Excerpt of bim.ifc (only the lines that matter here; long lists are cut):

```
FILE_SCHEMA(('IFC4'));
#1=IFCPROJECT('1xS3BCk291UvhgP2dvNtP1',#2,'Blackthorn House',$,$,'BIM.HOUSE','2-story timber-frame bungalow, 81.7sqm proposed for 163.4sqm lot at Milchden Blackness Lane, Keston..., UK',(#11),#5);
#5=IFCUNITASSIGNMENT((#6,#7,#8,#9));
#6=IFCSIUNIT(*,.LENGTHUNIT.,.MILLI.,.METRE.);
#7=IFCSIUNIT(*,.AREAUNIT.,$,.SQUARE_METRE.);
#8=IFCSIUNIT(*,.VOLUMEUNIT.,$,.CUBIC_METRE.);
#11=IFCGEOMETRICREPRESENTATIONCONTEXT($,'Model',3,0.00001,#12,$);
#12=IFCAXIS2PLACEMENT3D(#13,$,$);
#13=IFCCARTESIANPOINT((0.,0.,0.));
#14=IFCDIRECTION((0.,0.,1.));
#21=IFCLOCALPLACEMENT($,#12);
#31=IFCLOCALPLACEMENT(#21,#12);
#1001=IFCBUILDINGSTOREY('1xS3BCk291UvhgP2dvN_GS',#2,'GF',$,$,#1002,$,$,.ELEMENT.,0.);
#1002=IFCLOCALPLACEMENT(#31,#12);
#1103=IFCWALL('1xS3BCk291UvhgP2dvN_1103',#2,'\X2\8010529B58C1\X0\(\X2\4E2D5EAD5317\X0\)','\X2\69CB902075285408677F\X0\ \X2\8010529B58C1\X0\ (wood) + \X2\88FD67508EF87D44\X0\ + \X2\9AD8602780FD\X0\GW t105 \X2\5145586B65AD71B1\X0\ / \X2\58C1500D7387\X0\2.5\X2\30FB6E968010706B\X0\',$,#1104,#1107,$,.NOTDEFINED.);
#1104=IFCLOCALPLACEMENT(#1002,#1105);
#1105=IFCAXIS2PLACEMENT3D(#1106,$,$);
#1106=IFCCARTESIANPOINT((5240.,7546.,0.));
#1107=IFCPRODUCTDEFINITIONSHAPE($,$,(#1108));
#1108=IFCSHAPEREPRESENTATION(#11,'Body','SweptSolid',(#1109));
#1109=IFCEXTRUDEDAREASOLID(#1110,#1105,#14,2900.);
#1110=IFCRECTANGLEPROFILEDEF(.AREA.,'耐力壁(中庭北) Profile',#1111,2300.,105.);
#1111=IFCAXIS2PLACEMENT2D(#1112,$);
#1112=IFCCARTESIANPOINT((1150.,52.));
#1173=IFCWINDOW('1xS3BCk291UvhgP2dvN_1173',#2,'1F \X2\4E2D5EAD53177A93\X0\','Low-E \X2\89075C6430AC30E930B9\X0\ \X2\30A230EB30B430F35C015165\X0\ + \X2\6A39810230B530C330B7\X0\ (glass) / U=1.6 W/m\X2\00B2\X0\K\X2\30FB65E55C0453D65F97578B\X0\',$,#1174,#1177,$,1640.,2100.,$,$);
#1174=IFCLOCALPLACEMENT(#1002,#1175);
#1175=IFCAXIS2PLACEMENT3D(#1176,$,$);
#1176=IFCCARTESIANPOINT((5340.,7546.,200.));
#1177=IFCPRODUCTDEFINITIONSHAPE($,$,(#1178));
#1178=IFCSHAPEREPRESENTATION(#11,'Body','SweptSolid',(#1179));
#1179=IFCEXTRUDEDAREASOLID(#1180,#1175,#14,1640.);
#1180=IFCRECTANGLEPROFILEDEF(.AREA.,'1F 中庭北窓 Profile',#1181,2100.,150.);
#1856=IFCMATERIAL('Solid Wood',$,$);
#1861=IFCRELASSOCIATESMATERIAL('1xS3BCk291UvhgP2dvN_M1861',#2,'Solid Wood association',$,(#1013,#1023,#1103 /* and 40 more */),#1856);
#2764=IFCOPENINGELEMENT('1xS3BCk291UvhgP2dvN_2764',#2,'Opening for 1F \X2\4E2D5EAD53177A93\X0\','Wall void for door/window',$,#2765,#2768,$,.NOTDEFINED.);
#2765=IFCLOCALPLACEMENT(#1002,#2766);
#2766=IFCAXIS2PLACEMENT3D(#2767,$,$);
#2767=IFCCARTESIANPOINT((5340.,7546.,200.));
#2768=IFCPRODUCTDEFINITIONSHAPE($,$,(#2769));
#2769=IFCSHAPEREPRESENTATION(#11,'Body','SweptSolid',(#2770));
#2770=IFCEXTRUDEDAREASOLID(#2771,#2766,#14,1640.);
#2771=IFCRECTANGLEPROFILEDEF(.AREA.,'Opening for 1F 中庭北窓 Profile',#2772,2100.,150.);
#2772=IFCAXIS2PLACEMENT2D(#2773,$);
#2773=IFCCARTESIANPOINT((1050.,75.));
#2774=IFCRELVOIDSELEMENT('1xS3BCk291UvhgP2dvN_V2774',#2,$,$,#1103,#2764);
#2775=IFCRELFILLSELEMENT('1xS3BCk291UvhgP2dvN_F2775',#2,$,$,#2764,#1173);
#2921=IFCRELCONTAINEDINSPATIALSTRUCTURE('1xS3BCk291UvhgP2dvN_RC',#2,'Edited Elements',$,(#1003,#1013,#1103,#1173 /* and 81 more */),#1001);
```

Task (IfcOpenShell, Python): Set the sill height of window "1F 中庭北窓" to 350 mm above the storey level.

```python
import numpy as np
import ifcopenshell
import ifcopenshell.api.geometry
import ifcopenshell.geom
import ifcopenshell.util.element
import ifcopenshell.util.placement
import ifcopenshell.util.shape
import ifcopenshell.util.unit

model = ifcopenshell.open("bim.ifc")
unit_scale = ifcopenshell.util.unit.calculate_unit_scale(model)

window = model.by_id(1173)
opening = window.FillsVoids[0].RelatingOpeningElement
storey = ifcopenshell.util.element.get_container(window, ifc_class="IfcBuildingStorey")
level = ifcopenshell.util.placement.get_local_placement(storey.ObjectPlacement)[2, 3]

# The opening's origin need not be at the sill, so measure its lowest point.
shape = ifcopenshell.geom.create_shape(ifcopenshell.geom.settings(), opening)
bottom = ifcopenshell.util.shape.get_shape_bottom_elevation(shape, shape.geometry) / unit_scale
dz = level + 350.0 - bottom

shift = np.array([0.0, 0.0, dz])
# The window is not placed relative to its opening, so move both.
for product in (opening, window):
    matrix = ifcopenshell.util.placement.get_local_placement(product.ObjectPlacement)
    matrix[:3, 3] += shift
    ifcopenshell.api.geometry.edit_object_placement(model, product=product, matrix=matrix, is_si=False)

print(f"moved by {dz * unit_scale:+.3f} m")

model.write("bim_v2.ifc")
```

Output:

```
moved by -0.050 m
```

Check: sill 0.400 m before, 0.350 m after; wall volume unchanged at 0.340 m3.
